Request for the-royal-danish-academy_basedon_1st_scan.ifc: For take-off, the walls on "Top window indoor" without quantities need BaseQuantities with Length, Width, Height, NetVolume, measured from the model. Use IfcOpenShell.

First a look at what the model holds.

```python
import ifcopenshell
import ifcopenshell.util.element
import ifcopenshell.util.unit

model = ifcopenshell.open("the-royal-danish-academy_basedon_1st_scan.ifc")
print(model.schema)
for unit_type in ("LENGTHUNIT", "AREAUNIT", "VOLUMEUNIT"):
    print(unit_type, ifcopenshell.util.unit.calculate_unit_scale(model, unit_type))
storey = next(s for s in model.by_type("IfcBuildingStorey") if s.Name == "Top window indoor")
walls = [e for e in ifcopenshell.util.element.get_decomposition(storey) if e.is_a("IfcWall")]
for e in sorted(walls, key=lambda e: e.id()):
    print(e.id(), e.is_a(), e.Name, list(ifcopenshell.util.element.get_psets(e, qtos_only=True)), sep=" | ")
```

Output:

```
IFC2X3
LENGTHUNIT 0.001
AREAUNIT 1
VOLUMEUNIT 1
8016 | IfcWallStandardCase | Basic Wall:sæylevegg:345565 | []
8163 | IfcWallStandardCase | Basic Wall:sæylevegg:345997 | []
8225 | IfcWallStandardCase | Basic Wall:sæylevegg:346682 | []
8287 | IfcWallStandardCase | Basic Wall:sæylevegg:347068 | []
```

```python
import ifcopenshell
import ifcopenshell.api.pset
import ifcopenshell.geom
import ifcopenshell.util.element
import ifcopenshell.util.shape
import ifcopenshell.util.unit

model = ifcopenshell.open("the-royal-danish-academy_basedon_1st_scan.ifc")
unit_scale = ifcopenshell.util.unit.calculate_unit_scale(model)
volume_scale = ifcopenshell.util.unit.calculate_unit_scale(model, "VOLUMEUNIT")
settings = ifcopenshell.geom.settings()

storey = next(s for s in model.by_type("IfcBuildingStorey") if s.Name == "Top window indoor")
walls = [e for e in ifcopenshell.util.element.get_decomposition(storey) if e.is_a("IfcWall")]

for e in sorted(walls, key=lambda e: e.id()):
    if ifcopenshell.util.element.get_psets(e, qtos_only=True, should_inherit=False):
        continue
    # Geometry comes back in metres, in the element's own axes.
    shape = ifcopenshell.geom.create_shape(settings, e)
    values = {
        "Length": ifcopenshell.util.shape.get_x(shape.geometry) / unit_scale,
        "Width": ifcopenshell.util.shape.get_y(shape.geometry) / unit_scale,
        "Height": ifcopenshell.util.shape.get_z(shape.geometry) / unit_scale,
        "NetVolume": ifcopenshell.util.shape.get_volume(shape.geometry) / volume_scale,
    }
    qto = ifcopenshell.api.pset.add_qto(model, product=e, name="BaseQuantities")
    ifcopenshell.api.pset.edit_qto(model, qto=qto, properties=values)
    print(e.id(), {k: round(v, 3) for k, v in values.items()})

model.write("the-royal-danish-academy_basedon_1st_scan_edited.ifc")
```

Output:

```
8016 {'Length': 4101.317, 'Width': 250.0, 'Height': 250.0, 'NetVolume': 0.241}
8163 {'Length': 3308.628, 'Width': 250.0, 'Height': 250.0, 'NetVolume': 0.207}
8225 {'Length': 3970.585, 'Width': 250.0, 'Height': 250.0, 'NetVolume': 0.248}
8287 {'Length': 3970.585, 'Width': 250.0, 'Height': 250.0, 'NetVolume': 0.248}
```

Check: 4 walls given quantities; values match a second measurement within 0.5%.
